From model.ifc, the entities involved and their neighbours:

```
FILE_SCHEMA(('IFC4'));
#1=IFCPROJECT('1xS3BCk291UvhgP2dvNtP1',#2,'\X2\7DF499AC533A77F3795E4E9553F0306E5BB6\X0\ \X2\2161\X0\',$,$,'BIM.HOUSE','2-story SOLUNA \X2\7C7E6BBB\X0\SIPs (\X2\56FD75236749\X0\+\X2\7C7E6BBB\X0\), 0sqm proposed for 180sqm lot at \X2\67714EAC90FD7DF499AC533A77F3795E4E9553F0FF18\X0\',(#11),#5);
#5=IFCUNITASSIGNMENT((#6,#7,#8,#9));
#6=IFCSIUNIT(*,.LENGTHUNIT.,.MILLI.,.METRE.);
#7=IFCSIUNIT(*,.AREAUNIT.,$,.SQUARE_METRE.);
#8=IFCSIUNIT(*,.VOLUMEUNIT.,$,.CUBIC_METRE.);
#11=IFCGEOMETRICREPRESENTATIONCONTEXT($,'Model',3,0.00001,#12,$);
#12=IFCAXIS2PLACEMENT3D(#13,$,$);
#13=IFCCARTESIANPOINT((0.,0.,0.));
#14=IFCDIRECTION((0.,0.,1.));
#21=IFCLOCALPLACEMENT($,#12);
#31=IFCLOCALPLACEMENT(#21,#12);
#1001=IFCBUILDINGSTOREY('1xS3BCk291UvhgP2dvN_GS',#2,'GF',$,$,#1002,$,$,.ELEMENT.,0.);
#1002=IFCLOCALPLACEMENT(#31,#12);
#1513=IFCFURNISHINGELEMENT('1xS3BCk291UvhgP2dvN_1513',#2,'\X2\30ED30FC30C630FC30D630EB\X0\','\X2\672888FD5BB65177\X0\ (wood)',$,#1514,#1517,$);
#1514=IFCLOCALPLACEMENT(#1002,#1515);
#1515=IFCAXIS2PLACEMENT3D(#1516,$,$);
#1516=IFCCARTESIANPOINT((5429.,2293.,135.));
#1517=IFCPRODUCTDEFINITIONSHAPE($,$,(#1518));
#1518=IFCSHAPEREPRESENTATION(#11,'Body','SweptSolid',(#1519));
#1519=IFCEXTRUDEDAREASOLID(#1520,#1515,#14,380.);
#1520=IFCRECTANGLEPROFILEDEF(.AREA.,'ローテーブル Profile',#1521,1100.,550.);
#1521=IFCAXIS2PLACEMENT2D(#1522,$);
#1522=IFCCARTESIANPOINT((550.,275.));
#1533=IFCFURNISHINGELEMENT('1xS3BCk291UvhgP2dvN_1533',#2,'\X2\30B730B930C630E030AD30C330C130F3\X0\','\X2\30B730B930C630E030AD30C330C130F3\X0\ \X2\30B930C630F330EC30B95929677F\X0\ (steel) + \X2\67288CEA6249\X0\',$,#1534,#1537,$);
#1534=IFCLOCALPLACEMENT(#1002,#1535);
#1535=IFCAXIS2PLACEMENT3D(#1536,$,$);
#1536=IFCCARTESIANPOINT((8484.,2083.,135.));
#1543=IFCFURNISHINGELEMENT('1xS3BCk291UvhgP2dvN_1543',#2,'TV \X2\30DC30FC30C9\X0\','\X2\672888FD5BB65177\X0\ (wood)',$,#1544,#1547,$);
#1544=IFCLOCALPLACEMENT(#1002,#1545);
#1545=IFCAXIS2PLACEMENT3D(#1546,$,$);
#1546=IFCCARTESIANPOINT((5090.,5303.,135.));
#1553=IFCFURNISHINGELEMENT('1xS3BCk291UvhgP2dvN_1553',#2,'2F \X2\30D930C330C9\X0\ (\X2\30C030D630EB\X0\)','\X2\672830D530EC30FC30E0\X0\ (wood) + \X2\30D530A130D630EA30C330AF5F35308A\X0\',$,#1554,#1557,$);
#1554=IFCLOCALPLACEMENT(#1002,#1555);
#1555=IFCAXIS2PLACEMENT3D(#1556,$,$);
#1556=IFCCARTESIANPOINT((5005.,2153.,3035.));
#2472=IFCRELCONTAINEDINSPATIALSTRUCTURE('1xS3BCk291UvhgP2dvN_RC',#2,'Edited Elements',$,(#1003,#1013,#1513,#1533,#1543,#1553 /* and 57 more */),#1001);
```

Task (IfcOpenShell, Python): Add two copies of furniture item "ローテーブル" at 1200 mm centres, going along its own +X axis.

```python
import ifcopenshell
import ifcopenshell.api.geometry
import ifcopenshell.api.root
import ifcopenshell.util.element
import ifcopenshell.util.placement

model = ifcopenshell.open("model.ifc")


def reuse_history(source, copy):
    """copy_class also copies each property set's owner history, people and application; keep the originals."""
    for rel in copy.IsDefinedBy:
        if rel.is_a("IfcRelDefinesByProperties") and (history := rel.RelatingPropertyDefinition.OwnerHistory):
            rel.RelatingPropertyDefinition.OwnerHistory = source.OwnerHistory
            ifcopenshell.util.element.remove_deep2(model, history)


source = model.by_guid("1xS3BCk291UvhgP2dvN_1513")
base = ifcopenshell.util.placement.get_local_placement(source.ObjectPlacement)
step = base[:3, 0] * 1200.0

for i in range(1, 3):
    copy = ifcopenshell.api.root.copy_class(model, product=source)
    copy.Representation = ifcopenshell.util.element.copy_deep(
        model, source.Representation, exclude=["IfcGeometricRepresentationContext", "IfcRepresentationMap"]
    )
    reuse_history(source, copy)
    matrix = base.copy()
    matrix[:3, 3] += i * step
    print("added at", matrix[:3, 3].round(3) + 0.0)
    ifcopenshell.api.geometry.edit_object_placement(model, product=copy, matrix=matrix, is_si=False)

model.write("model_rev.ifc")
```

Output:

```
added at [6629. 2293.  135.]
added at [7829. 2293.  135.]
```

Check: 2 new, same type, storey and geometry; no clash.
